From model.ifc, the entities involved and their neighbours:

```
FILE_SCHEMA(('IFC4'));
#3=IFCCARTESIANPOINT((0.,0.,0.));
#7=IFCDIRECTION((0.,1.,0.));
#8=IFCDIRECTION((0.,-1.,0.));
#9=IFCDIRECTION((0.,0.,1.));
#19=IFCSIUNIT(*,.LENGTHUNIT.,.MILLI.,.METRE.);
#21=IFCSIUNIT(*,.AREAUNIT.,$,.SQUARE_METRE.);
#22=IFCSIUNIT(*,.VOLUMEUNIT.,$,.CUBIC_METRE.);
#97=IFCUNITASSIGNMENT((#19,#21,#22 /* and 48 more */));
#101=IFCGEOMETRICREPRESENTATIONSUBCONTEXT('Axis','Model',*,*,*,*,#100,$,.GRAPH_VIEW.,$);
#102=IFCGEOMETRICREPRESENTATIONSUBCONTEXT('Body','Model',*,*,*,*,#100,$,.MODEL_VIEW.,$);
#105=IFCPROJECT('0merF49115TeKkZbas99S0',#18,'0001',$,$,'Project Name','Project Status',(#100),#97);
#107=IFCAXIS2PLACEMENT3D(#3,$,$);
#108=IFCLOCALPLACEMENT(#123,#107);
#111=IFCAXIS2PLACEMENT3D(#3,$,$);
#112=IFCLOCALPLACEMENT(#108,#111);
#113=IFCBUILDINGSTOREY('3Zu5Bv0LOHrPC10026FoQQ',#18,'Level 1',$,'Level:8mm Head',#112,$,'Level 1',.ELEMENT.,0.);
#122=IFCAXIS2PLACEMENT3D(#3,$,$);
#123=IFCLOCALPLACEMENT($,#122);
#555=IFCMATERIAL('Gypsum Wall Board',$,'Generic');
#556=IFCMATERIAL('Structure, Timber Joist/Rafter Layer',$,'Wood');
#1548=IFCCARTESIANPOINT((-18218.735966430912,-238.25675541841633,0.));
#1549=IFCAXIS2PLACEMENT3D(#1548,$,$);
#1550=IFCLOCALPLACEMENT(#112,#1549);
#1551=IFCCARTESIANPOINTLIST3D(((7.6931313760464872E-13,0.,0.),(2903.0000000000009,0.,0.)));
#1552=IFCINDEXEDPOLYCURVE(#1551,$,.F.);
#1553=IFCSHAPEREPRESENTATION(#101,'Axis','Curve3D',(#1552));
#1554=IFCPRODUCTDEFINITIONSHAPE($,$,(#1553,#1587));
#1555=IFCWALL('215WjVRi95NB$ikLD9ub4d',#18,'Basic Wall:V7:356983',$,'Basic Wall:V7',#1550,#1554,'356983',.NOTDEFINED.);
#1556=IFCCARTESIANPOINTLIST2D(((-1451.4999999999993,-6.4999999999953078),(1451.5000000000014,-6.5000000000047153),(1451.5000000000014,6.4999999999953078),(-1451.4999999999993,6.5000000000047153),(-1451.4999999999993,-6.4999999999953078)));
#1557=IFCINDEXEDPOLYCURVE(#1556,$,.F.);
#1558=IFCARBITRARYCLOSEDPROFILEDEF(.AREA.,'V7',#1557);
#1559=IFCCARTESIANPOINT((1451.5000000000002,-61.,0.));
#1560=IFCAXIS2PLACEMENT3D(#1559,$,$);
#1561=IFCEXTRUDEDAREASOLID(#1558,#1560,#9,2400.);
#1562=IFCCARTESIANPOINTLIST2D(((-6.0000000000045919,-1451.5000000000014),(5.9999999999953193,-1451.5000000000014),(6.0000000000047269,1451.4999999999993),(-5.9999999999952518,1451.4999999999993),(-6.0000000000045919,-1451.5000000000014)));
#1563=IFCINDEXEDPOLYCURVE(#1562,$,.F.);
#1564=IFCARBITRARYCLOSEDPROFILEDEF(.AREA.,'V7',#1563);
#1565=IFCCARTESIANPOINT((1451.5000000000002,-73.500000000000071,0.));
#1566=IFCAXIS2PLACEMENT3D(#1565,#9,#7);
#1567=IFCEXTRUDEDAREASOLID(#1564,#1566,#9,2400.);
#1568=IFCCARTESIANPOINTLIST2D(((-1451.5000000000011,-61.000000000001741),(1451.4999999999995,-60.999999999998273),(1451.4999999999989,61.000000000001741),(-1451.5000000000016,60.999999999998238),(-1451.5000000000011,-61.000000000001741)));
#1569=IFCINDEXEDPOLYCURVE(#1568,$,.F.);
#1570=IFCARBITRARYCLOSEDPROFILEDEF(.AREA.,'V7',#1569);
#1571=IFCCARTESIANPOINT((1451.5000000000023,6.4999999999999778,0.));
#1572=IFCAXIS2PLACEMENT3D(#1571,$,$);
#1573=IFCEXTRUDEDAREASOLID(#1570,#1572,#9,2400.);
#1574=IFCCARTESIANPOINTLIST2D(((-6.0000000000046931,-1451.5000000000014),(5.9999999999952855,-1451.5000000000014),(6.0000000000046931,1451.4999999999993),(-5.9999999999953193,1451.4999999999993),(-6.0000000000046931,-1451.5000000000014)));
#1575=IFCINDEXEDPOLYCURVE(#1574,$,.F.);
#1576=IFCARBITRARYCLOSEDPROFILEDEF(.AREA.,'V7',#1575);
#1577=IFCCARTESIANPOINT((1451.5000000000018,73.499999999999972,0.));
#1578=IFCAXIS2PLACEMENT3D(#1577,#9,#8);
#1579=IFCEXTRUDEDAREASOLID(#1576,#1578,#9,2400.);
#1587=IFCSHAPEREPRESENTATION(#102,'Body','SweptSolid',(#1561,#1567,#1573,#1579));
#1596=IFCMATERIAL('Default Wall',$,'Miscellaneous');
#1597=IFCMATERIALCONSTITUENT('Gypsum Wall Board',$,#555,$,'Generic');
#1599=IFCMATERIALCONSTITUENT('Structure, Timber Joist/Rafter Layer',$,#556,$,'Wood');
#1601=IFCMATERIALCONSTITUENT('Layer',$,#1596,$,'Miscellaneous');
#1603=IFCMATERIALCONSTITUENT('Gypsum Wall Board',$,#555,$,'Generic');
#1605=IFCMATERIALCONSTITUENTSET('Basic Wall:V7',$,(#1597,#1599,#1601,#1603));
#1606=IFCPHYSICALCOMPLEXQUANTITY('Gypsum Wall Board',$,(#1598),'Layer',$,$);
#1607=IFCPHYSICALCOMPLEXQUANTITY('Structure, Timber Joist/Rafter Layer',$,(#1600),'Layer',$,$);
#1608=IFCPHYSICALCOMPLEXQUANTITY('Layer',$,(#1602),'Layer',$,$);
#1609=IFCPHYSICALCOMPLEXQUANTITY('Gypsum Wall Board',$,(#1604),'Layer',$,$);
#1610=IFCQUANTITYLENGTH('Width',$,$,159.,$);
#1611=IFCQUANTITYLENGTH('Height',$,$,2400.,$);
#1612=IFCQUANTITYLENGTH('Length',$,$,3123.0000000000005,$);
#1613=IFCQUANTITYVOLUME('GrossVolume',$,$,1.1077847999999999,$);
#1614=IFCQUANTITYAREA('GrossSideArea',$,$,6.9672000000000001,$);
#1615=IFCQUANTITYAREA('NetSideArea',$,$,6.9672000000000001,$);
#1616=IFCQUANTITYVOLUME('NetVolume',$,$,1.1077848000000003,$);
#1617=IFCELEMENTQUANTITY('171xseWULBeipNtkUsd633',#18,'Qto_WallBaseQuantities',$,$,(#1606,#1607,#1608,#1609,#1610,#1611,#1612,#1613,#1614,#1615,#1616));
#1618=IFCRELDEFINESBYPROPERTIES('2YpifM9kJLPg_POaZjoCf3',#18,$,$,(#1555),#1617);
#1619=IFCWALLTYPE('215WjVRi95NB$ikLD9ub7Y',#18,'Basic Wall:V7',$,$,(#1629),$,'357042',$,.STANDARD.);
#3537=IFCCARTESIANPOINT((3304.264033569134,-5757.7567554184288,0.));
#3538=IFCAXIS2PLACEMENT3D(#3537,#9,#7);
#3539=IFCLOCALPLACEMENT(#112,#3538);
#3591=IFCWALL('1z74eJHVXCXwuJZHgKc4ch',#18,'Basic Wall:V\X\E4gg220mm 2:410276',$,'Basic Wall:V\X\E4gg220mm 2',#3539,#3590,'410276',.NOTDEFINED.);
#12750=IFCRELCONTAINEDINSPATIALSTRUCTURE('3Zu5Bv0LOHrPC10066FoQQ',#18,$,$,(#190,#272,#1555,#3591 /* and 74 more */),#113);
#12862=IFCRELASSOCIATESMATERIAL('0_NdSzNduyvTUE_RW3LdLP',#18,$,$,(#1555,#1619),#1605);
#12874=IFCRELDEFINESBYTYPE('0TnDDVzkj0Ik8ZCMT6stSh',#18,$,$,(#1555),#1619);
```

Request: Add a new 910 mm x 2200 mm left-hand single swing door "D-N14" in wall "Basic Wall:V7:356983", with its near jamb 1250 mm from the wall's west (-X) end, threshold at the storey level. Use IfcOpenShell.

```python
import numpy as np
import ifcopenshell
import ifcopenshell.api.feature
import ifcopenshell.api.geometry
import ifcopenshell.api.pset
import ifcopenshell.api.root
import ifcopenshell.api.spatial
import ifcopenshell.geom
import ifcopenshell.util.element
import ifcopenshell.util.placement
import ifcopenshell.util.representation
import ifcopenshell.util.shape
import ifcopenshell.util.unit

model = ifcopenshell.open("model.ifc")
unit_scale = ifcopenshell.util.unit.calculate_unit_scale(model)
area_scale = ifcopenshell.util.unit.calculate_unit_scale(model, "AREAUNIT")
volume_scale = ifcopenshell.util.unit.calculate_unit_scale(model, "VOLUMEUNIT")
settings = ifcopenshell.geom.settings()


def volume(element):
    """Net volume in cubic metres, openings subtracted."""
    shape = ifcopenshell.geom.create_shape(settings, element)
    return ifcopenshell.util.shape.get_volume(shape.geometry)


wall = model.by_id(1555)
storey = ifcopenshell.util.element.get_container(wall, ifc_class="IfcBuildingStorey")
context = ifcopenshell.util.representation.get_context(model, "Model", "Body", "MODEL_VIEW")
before = volume(wall)

width, height, from_end, sill = 0.91, 2.2, 1.25, 0.0  # metres

# The wall runs along its own X axis, and the end named is its -X end.
wall_shape = ifcopenshell.geom.create_shape(settings, wall)
x, y, z = ifcopenshell.util.shape.get_vertices(wall_shape.geometry).T
start = x.min() + from_end
face, thickness = float(y.min()), float(y.max() - y.min())
wall_matrix = ifcopenshell.util.placement.get_local_placement(wall.ObjectPlacement)
level = ifcopenshell.util.placement.get_local_placement(storey.ObjectPlacement)[2, 3]


def in_wall(x, y):
    """Placement at x, y metres in the wall's axes, at sill height."""
    matrix = wall_matrix.copy()
    matrix[:, 3] = wall_matrix @ np.array([x / unit_scale, y / unit_scale, 0.0, 1.0])
    matrix[2, 3] = level + sill / unit_scale
    return matrix


# Opening: a box that overshoots both wall faces by 50 mm.
opening = ifcopenshell.api.root.create_entity(model, ifc_class="IfcOpeningElement", predefined_type="OPENING")
box = ifcopenshell.api.geometry.add_wall_representation(
    model, context=context, length=width, height=height, thickness=thickness + 0.1
)
ifcopenshell.api.geometry.assign_representation(model, product=opening, representation=box)
ifcopenshell.api.geometry.edit_object_placement(model, product=opening, matrix=in_wall(start, face - 0.05), is_si=False)
ifcopenshell.api.feature.add_feature(model, feature=opening, element=wall)

door = ifcopenshell.api.root.create_entity(model, ifc_class="IfcDoor", name="D-N14", predefined_type="DOOR")
door.OverallWidth, door.OverallHeight = width / unit_scale, height / unit_scale
door.OperationType = "SINGLE_SWING_LEFT"
body = ifcopenshell.api.geometry.add_door_representation(
    model,
    context=context,
    overall_width=door.OverallWidth,
    overall_height=door.OverallHeight,
    operation_type="SINGLE_SWING_LEFT",
    lining_properties={"LiningDepth": thickness / unit_scale, "ThresholdDepth": thickness / unit_scale},
)
ifcopenshell.api.geometry.assign_representation(model, product=door, representation=body)
ifcopenshell.api.spatial.assign_container(model, products=[door], relating_structure=storey)
ifcopenshell.api.feature.add_filling(model, opening=opening, element=door)

# The lining spans the wall, so the door starts at the wall face.
ifcopenshell.api.geometry.edit_object_placement(model, product=door, matrix=in_wall(start, face), is_si=False)

after = volume(wall)

# Update the wall's stored quantities.
qto = model.by_id(ifcopenshell.util.element.get_pset(wall, "Qto_WallBaseQuantities", should_inherit=False)["id"])
ifcopenshell.api.pset.edit_qto(model, qto=qto, properties={
    "NetSideArea": after / thickness / area_scale,
    "NetVolume": after / volume_scale,
})

print(f"wall volume {before:.3f} -> {after:.3f} m3")

model.write("model_rev.ifc")
```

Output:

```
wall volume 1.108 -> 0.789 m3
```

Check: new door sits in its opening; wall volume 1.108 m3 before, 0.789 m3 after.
